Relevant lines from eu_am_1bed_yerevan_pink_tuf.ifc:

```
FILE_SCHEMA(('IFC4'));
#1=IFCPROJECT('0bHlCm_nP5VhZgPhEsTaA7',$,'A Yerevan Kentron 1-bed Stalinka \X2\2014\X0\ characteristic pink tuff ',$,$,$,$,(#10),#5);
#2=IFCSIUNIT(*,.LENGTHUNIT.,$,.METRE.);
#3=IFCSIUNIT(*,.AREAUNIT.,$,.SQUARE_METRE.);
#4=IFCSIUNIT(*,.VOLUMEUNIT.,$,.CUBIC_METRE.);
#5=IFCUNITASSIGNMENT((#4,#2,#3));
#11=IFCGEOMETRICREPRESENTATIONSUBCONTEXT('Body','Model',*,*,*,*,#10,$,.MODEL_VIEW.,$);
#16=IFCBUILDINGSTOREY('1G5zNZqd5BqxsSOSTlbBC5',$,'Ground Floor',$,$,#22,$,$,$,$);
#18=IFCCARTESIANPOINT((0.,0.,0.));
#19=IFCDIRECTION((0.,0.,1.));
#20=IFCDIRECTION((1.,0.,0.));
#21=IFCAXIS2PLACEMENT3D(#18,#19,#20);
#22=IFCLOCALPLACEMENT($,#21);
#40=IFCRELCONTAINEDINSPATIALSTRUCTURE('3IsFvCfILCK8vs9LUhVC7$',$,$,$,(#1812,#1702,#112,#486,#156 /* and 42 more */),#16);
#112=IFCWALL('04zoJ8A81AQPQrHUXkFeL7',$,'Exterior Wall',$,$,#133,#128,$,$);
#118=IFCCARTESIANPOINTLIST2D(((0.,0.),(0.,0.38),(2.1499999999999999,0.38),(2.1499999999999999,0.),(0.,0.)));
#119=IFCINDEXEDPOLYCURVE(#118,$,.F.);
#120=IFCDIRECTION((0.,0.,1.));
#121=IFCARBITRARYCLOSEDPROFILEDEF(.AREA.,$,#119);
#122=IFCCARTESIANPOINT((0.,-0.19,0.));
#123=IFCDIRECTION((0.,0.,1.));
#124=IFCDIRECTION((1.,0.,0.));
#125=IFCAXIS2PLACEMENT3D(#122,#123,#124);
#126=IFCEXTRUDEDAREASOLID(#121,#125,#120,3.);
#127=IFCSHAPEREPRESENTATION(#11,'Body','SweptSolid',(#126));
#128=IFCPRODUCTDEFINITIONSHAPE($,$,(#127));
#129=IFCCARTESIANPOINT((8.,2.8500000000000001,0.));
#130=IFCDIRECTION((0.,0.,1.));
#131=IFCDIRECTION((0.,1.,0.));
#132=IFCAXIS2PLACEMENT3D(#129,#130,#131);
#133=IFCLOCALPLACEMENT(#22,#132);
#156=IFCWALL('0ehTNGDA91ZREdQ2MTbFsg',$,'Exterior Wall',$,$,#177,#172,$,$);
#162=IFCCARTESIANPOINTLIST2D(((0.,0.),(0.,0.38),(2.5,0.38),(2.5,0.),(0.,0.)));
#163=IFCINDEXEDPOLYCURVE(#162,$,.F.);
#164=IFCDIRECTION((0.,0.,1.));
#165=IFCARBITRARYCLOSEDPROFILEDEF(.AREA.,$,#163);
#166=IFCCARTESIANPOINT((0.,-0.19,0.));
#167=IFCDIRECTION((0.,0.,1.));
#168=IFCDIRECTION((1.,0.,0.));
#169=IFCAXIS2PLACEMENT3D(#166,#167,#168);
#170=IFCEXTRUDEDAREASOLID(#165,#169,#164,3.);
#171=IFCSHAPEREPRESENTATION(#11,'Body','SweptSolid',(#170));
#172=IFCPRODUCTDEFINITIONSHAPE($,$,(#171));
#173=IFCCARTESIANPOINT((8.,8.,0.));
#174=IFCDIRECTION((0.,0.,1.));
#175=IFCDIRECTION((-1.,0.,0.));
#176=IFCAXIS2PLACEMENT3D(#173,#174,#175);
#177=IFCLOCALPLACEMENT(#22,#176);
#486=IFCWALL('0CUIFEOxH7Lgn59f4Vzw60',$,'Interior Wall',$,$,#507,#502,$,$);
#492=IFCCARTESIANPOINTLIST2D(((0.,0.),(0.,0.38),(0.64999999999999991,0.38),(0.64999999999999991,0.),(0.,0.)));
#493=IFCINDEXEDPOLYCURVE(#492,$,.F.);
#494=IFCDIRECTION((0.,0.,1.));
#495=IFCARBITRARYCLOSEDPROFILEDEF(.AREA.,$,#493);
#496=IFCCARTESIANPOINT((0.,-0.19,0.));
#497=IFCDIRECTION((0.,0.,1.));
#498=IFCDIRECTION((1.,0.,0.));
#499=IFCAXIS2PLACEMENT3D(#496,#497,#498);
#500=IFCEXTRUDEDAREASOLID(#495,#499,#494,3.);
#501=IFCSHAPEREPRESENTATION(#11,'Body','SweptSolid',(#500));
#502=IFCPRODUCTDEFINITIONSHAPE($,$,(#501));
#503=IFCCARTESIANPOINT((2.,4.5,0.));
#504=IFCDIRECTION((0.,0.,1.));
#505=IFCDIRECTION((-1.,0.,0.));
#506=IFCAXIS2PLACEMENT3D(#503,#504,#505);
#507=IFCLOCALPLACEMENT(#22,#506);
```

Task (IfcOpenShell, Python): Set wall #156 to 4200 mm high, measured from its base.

```python
import ifcopenshell
import ifcopenshell.geom
import ifcopenshell.util.representation
import ifcopenshell.util.shape
import ifcopenshell.util.unit

model = ifcopenshell.open("eu_am_1bed_yerevan_pink_tuf.ifc")
unit_scale = ifcopenshell.util.unit.calculate_unit_scale(model)
settings = ifcopenshell.geom.settings()


def volume(element):
    """Net volume in cubic metres, openings subtracted."""
    shape = ifcopenshell.geom.create_shape(settings, element)
    return ifcopenshell.util.shape.get_volume(shape.geometry)


wall = model.by_guid("0ehTNGDA91ZREdQ2MTbFsg")
before = volume(wall)

body = ifcopenshell.util.representation.get_representation(wall, "Model", "Body")
solid = body.Items[0]
old_height = solid.Depth
solid.Depth = 4.2 / unit_scale
after = volume(wall)

print(f"height {old_height:g} -> {solid.Depth:g}, volume {before:.3f} -> {after:.3f} m3")

model.write("eu_am_1bed_yerevan_pink_tuf_v2.ifc")
```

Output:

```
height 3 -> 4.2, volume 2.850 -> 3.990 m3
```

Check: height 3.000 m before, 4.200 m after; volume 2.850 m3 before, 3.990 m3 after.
